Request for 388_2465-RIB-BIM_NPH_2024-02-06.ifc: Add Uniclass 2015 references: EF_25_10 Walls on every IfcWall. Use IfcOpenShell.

First a look at what the model holds.

```python
import ifcopenshell

model = ifcopenshell.open("388_2465-RIB-BIM_NPH_2024-02-06.ifc")
print(model.schema)
print("classifications:", [c.Name for c in model.by_type("IfcClassification")])
for ifc_class in ("IfcDoor", "IfcRoof", "IfcStair", "IfcWall", "IfcWindow"):
    print(ifc_class, len(model.by_type(ifc_class)))
```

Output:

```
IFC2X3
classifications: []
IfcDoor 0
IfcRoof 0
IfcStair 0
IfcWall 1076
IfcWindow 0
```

```python
import ifcopenshell
import ifcopenshell.api.classification

model = ifcopenshell.open("388_2465-RIB-BIM_NPH_2024-02-06.ifc")

# IFC2X3 requires Source and Edition and has no link from the project to the system.
system = model.create_entity("IfcClassification", Source="NBS", Edition="2015", Name="Uniclass 2015")

codes = {
    "IfcWall": ("EF_25_10", "Walls"),
}
for ifc_class, (code, name) in codes.items():
    products = model.by_type(ifc_class)
    ifcopenshell.api.classification.add_reference(
        model, products=products, classification=system, identification=code, name=name
    )
    print(code, len(products))

model.write("388_2465-RIB-BIM_NPH_2024-02-06_updated.ifc")
```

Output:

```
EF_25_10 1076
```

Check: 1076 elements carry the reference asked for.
